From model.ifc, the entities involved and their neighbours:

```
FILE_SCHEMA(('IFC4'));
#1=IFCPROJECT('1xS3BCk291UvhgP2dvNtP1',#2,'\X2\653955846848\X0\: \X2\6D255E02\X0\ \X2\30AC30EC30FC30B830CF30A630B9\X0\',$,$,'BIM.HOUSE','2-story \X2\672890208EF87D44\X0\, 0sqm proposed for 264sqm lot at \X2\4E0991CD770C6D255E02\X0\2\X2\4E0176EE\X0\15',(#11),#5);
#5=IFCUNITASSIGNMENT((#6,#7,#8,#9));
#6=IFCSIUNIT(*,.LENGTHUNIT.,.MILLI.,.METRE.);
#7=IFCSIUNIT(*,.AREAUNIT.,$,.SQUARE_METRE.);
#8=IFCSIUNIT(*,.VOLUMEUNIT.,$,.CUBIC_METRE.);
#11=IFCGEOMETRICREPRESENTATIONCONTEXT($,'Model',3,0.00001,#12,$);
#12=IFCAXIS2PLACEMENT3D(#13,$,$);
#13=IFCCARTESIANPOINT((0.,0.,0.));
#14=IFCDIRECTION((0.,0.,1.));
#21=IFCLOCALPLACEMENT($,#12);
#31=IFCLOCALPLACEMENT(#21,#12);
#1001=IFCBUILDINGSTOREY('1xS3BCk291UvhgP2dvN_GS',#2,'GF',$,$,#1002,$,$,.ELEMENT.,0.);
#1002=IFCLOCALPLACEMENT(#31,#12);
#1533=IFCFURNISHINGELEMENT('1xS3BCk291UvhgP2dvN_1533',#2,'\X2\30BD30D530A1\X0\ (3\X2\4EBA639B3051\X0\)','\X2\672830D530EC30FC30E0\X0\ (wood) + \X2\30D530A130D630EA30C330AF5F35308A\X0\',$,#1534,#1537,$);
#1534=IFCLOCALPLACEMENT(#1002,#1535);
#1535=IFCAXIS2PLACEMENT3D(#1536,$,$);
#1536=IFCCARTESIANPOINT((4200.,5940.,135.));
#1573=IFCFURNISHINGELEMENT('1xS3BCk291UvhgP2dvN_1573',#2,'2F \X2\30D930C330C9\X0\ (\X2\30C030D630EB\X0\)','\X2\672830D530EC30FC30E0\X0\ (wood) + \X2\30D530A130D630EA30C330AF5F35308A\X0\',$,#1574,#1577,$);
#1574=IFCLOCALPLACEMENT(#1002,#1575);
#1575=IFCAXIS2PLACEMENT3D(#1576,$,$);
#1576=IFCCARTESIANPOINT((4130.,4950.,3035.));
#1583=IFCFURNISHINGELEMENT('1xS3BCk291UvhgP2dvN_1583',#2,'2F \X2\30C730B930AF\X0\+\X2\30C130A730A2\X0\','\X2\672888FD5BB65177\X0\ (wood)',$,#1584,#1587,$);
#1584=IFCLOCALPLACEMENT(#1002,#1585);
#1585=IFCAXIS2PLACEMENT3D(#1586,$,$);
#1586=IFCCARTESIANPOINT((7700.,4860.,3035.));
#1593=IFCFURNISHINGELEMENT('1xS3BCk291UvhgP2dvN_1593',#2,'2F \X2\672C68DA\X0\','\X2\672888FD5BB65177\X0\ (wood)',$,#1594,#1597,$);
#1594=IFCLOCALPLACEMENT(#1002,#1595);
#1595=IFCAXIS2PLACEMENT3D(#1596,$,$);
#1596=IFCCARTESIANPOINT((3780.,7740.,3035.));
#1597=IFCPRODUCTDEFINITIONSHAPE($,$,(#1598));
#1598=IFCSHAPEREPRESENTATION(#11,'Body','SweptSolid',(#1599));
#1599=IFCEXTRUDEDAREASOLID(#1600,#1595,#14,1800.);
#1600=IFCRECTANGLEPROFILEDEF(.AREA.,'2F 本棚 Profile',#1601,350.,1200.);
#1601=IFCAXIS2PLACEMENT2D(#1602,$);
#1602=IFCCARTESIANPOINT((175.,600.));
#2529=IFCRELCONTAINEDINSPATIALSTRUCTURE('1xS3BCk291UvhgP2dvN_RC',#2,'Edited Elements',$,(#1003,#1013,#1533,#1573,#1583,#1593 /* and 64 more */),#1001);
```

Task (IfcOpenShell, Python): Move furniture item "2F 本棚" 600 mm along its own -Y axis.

```python
import ifcopenshell
import ifcopenshell.api.geometry
import ifcopenshell.util.placement
import ifcopenshell.util.unit

model = ifcopenshell.open("model.ifc")
unit_scale = ifcopenshell.util.unit.calculate_unit_scale(model)

item = model.by_guid("1xS3BCk291UvhgP2dvN_1593")
matrix = ifcopenshell.util.placement.get_local_placement(item.ObjectPlacement)
matrix[:3, 3] -= matrix[:3, 1] * 0.6 / unit_scale
ifcopenshell.api.geometry.edit_object_placement(model, product=item, matrix=matrix, is_si=False)

print(ifcopenshell.util.placement.get_local_placement(item.ObjectPlacement).round(3) + 0.0)

model.write("model_rev.ifc")
```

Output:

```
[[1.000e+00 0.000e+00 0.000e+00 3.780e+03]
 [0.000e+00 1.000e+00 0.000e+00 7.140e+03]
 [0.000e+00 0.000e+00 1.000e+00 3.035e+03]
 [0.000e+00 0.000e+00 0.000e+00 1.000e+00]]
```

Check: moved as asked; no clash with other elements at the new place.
